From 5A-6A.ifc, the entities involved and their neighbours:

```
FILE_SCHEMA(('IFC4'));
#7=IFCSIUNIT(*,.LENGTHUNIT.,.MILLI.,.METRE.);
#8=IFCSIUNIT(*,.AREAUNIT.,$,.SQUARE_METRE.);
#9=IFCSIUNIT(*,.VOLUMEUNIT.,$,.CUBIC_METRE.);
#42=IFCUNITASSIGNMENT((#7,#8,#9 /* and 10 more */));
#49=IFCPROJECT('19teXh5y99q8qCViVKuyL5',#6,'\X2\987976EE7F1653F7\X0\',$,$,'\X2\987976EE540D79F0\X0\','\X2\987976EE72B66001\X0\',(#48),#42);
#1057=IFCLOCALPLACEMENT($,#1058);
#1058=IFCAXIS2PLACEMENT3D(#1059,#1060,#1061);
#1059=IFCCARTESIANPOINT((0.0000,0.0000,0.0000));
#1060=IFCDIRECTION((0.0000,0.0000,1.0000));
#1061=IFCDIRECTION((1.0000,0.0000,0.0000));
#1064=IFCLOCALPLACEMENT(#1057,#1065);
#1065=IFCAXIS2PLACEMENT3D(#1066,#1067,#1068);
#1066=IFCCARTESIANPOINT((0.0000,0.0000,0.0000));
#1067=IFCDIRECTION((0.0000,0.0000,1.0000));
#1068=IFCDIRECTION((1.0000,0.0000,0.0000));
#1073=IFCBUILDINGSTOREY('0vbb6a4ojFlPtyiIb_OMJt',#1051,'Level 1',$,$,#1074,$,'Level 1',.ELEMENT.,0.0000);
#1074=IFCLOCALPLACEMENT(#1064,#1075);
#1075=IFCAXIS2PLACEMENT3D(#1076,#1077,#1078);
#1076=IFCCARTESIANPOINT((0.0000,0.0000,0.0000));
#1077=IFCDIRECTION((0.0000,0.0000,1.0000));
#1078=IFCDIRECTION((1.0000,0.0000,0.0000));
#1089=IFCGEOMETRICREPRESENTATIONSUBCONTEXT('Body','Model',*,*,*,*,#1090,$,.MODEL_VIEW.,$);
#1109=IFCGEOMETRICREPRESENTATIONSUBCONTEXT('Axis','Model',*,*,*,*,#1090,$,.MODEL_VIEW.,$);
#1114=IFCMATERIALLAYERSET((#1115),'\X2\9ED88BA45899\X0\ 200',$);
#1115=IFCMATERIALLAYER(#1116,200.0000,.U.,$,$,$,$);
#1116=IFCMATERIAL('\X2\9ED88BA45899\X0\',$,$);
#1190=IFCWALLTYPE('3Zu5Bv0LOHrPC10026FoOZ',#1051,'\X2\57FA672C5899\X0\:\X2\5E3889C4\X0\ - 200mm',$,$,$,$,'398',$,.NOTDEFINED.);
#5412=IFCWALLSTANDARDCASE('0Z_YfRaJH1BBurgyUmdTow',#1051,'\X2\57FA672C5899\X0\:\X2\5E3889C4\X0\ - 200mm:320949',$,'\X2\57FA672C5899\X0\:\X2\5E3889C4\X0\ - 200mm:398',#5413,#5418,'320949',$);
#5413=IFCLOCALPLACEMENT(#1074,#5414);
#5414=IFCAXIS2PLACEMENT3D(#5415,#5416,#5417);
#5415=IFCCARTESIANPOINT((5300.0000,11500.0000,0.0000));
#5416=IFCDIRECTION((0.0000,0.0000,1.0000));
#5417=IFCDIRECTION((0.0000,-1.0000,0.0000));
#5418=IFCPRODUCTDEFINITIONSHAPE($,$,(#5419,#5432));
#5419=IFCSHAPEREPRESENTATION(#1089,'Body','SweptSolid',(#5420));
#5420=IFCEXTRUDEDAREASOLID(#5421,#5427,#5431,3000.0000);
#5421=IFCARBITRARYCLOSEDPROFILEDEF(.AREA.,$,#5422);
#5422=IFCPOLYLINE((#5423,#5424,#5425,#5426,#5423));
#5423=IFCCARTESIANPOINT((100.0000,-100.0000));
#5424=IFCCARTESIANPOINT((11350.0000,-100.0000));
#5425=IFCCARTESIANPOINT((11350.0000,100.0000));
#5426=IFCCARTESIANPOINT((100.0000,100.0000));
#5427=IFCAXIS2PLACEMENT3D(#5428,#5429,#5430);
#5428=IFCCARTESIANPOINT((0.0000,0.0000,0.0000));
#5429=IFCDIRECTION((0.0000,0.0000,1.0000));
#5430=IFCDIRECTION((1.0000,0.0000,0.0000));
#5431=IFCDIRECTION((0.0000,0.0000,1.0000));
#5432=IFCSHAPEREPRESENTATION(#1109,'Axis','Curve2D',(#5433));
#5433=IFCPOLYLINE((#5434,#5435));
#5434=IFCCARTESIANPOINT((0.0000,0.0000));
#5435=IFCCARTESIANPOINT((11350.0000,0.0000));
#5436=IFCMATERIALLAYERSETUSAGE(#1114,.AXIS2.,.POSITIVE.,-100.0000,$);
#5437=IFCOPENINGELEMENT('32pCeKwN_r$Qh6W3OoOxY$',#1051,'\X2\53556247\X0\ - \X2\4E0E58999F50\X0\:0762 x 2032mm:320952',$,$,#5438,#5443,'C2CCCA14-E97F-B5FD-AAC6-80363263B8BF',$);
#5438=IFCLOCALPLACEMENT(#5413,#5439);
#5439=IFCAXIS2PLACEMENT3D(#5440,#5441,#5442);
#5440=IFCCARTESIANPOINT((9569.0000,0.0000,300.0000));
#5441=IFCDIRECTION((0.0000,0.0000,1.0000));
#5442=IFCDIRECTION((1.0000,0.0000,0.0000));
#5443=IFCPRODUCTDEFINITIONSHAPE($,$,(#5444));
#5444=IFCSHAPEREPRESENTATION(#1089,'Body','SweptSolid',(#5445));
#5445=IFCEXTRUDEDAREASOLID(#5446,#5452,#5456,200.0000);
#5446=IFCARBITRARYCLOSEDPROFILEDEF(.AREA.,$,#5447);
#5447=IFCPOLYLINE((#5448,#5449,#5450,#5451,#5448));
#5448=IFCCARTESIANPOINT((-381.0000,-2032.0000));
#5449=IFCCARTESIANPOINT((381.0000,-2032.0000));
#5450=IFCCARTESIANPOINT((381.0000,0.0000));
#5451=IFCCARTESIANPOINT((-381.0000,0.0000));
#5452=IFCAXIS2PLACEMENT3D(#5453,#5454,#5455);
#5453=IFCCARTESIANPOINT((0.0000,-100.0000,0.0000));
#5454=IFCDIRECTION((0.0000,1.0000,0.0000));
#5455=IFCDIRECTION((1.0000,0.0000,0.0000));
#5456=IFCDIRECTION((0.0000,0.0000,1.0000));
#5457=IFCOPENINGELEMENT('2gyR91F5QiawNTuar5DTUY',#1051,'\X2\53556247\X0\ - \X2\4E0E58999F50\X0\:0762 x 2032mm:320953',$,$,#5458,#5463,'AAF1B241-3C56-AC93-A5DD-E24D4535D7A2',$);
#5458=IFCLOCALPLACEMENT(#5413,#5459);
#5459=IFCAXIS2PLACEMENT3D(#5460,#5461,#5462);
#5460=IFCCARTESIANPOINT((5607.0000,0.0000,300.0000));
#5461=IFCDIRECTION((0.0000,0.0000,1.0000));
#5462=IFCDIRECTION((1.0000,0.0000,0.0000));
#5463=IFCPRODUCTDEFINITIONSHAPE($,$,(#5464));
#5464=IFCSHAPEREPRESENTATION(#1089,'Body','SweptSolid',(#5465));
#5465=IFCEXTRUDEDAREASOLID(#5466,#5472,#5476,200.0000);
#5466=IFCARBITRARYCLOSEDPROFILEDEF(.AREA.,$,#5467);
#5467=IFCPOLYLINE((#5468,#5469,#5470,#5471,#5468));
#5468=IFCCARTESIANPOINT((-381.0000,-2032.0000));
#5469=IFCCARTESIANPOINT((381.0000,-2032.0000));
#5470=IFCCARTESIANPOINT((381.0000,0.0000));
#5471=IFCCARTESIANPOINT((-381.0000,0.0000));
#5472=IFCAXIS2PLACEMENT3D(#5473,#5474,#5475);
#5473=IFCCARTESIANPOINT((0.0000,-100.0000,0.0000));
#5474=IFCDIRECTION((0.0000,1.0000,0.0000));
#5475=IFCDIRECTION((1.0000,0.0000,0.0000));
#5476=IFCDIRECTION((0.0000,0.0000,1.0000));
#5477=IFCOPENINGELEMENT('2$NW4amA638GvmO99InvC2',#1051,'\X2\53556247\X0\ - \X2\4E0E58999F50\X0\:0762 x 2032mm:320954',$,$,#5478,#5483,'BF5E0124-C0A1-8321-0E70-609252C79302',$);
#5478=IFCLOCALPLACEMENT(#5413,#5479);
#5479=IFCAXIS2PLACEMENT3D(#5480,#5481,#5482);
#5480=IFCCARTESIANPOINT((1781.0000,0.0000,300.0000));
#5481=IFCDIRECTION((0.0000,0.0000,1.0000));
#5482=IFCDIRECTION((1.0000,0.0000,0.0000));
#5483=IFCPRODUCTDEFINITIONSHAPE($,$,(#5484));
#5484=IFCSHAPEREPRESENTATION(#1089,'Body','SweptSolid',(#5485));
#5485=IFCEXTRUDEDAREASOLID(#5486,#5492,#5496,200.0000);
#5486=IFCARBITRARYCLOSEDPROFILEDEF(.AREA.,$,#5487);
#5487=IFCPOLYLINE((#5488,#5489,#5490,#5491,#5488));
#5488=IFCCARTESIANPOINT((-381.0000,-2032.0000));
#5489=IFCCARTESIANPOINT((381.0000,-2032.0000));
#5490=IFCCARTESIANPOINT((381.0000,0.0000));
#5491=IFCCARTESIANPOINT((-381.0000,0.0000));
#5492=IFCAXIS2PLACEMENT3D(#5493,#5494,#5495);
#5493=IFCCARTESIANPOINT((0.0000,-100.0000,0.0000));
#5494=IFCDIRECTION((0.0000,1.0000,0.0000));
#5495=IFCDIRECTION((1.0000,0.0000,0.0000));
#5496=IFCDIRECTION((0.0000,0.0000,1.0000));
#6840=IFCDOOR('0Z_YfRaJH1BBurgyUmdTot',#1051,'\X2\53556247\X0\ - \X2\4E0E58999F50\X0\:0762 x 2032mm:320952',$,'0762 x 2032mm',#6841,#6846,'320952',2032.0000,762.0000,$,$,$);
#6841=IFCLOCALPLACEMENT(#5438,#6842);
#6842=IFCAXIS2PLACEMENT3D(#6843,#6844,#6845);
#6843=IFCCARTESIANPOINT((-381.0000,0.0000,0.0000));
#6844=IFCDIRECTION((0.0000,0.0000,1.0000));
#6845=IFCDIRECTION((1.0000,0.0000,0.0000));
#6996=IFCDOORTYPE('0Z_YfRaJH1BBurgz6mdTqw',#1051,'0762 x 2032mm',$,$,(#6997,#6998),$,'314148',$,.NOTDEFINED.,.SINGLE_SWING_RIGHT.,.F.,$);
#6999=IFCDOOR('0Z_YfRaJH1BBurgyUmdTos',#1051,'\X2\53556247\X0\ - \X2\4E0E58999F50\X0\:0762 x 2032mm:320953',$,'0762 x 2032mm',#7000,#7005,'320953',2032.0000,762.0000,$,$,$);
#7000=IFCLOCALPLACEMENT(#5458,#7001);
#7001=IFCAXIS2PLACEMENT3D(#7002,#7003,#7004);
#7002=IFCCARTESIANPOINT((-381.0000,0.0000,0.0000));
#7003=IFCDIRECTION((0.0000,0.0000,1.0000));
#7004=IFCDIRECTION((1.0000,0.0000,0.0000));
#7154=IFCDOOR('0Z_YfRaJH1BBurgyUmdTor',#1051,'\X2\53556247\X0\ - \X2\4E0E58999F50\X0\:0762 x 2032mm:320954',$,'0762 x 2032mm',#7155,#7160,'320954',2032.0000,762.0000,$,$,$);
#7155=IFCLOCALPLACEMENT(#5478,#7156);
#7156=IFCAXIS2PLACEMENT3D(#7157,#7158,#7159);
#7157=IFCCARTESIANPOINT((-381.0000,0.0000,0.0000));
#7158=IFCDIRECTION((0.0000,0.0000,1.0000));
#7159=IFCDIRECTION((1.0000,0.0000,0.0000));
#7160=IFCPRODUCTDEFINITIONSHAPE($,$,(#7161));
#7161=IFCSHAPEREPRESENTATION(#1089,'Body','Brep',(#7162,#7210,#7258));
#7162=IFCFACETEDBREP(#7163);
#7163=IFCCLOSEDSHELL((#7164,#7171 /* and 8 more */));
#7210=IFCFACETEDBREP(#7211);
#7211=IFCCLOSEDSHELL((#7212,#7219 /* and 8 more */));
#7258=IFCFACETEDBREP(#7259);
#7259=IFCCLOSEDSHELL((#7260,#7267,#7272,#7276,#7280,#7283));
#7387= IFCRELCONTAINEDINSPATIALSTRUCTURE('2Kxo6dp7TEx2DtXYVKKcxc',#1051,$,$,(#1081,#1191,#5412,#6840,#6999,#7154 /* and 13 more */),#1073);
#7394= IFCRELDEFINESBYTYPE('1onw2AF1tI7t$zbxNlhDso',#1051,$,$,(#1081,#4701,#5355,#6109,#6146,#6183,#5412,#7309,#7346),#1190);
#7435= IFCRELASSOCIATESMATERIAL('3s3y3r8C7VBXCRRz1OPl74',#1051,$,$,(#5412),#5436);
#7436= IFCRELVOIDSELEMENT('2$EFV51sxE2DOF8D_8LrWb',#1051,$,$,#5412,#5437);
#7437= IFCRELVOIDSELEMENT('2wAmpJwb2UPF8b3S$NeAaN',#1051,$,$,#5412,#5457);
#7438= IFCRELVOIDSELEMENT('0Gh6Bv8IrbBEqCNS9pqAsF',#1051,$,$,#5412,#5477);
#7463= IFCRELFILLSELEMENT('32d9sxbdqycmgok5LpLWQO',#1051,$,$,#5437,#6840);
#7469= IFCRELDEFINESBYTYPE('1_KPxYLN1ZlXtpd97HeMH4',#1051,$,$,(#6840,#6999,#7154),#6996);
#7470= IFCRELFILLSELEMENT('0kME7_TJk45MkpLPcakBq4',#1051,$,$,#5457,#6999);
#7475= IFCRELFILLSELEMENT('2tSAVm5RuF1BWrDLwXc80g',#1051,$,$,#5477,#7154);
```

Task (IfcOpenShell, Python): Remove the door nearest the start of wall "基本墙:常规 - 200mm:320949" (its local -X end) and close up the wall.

```python
import ifcopenshell
import ifcopenshell.api.feature
import ifcopenshell.api.root
import ifcopenshell.geom
import ifcopenshell.util.shape

model = ifcopenshell.open("5A-6A.ifc")
settings = ifcopenshell.geom.settings()


def volume(element):
    """Net volume in cubic metres, openings subtracted."""
    shape = ifcopenshell.geom.create_shape(settings, element)
    return ifcopenshell.util.shape.get_volume(shape.geometry)


door = model.by_guid("0Z_YfRaJH1BBurgyUmdTor")
opening = door.FillsVoids[0].RelatingOpeningElement
wall = opening.VoidsElements[0].RelatingBuildingElement
before = volume(wall)

ifcopenshell.api.root.remove_product(model, product=door)
ifcopenshell.api.feature.remove_feature(model, feature=opening)

after = volume(wall)

print(f"wall volume {before:.3f} -> {after:.3f} m3")

model.write("5A-6A_rev.ifc")
```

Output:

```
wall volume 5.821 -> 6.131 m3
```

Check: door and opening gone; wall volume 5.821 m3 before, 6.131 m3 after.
